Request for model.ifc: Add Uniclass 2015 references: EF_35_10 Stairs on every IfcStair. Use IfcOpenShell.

First a look at what the model holds.

```python
import ifcopenshell

model = ifcopenshell.open("model.ifc")
print(model.schema)
print("classifications:", [c.Name for c in model.by_type("IfcClassification")])
for ifc_class in ("IfcDoor", "IfcRoof", "IfcStair", "IfcWall", "IfcWindow"):
    print(ifc_class, len(model.by_type(ifc_class)))
```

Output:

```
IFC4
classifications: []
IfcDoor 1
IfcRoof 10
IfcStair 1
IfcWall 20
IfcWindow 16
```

```python
import ifcopenshell
import ifcopenshell.api.classification

model = ifcopenshell.open("model.ifc")

system = ifcopenshell.api.classification.add_classification(model, classification="Uniclass 2015")

codes = {
    "IfcStair": ("EF_35_10", "Stairs"),
}
for ifc_class, (code, name) in codes.items():
    products = model.by_type(ifc_class)
    ifcopenshell.api.classification.add_reference(
        model, products=products, classification=system, identification=code, name=name
    )
    print(code, len(products))

model.write("model_updated.ifc")
```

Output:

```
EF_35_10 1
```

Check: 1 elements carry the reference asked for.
